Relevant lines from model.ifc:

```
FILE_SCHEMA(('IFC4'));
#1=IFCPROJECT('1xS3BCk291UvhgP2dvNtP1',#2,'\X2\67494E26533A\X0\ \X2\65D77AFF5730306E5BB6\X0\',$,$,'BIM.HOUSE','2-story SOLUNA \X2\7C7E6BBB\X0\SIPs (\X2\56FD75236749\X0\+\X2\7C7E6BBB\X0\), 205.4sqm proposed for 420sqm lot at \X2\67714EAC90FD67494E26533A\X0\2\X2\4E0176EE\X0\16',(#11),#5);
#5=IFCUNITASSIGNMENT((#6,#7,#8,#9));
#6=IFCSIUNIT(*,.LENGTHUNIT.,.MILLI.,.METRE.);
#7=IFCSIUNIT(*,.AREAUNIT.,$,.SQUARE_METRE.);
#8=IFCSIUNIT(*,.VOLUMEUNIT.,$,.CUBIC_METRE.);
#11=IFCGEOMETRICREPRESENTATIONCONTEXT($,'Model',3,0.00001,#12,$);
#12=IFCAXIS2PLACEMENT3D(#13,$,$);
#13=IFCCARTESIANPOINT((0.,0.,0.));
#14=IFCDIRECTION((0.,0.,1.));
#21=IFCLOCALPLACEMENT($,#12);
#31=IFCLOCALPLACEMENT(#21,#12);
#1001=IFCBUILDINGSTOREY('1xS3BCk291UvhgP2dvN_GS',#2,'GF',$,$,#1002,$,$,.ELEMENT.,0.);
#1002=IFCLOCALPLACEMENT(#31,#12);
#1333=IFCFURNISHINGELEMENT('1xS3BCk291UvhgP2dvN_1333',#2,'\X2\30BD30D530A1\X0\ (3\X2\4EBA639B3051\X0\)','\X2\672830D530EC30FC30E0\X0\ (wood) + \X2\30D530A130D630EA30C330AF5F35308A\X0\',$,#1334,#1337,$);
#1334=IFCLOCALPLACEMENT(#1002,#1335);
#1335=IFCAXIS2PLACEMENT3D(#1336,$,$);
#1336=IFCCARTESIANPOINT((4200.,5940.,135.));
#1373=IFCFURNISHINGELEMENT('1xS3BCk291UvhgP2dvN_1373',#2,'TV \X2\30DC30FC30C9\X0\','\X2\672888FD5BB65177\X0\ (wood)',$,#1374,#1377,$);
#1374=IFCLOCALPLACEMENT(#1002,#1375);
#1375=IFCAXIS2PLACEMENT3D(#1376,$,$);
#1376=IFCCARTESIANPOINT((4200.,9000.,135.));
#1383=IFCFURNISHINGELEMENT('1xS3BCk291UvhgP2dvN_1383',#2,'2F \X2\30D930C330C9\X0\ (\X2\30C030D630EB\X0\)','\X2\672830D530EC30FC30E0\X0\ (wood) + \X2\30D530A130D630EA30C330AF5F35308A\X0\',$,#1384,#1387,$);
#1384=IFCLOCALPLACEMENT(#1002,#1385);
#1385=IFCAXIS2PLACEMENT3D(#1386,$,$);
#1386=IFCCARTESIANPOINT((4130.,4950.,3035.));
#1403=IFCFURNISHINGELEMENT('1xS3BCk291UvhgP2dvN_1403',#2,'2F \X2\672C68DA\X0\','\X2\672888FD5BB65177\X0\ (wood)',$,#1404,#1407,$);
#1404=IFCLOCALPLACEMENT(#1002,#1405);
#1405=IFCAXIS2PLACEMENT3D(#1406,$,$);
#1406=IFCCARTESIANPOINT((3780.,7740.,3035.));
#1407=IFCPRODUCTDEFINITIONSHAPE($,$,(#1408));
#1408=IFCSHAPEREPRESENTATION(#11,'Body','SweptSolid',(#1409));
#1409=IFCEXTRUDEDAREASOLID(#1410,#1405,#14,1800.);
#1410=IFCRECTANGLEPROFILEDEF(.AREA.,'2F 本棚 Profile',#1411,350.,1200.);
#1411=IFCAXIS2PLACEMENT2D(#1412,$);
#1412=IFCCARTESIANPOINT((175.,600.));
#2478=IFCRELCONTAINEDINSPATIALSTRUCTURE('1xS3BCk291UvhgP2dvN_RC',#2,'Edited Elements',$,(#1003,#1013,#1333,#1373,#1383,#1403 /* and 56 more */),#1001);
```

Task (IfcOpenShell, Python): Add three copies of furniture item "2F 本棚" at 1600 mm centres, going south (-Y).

```python
import numpy as np
import ifcopenshell
import ifcopenshell.api.geometry
import ifcopenshell.api.root
import ifcopenshell.util.element
import ifcopenshell.util.placement

model = ifcopenshell.open("model.ifc")


def reuse_history(source, copy):
    """copy_class also copies each property set's owner history, people and application; keep the originals."""
    for rel in copy.IsDefinedBy:
        if rel.is_a("IfcRelDefinesByProperties") and (history := rel.RelatingPropertyDefinition.OwnerHistory):
            rel.RelatingPropertyDefinition.OwnerHistory = source.OwnerHistory
            ifcopenshell.util.element.remove_deep2(model, history)


source = model.by_guid("1xS3BCk291UvhgP2dvN_1403")
base = ifcopenshell.util.placement.get_local_placement(source.ObjectPlacement)
step = np.array([0.0, -1.0, 0.0]) * 1600.0

for i in range(1, 4):
    copy = ifcopenshell.api.root.copy_class(model, product=source)
    copy.Representation = ifcopenshell.util.element.copy_deep(
        model, source.Representation, exclude=["IfcGeometricRepresentationContext", "IfcRepresentationMap"]
    )
    reuse_history(source, copy)
    matrix = base.copy()
    matrix[:3, 3] += i * step
    print("added at", matrix[:3, 3].round(3) + 0.0)
    ifcopenshell.api.geometry.edit_object_placement(model, product=copy, matrix=matrix, is_si=False)

model.write("model-out.ifc")
```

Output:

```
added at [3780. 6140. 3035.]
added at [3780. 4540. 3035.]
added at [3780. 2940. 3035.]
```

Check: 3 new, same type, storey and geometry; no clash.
